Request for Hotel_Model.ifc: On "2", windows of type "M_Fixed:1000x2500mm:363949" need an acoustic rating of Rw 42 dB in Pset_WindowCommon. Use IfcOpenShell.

First a look at what the model holds.

```python
import ifcopenshell
import ifcopenshell.util.element

model = ifcopenshell.open("Hotel_Model.ifc")
print(model.schema)
storey = next(s for s in model.by_type("IfcBuildingStorey") if s.Name == "2")
windows = [e for e in ifcopenshell.util.element.get_decomposition(storey) if e.is_a("IfcWindow")]
seen = {}
for e in windows:
    element_type = ifcopenshell.util.element.get_type(e)
    key = (element_type.Name if element_type != e and element_type else None, ifcopenshell.util.element.get_pset(e, "Pset_WindowCommon", "AcousticRating"))
    seen[key] = seen.get(key, 0) + 1
for (name, value), count in sorted(seen.items(), key=str):
    print(count, "x", name, "|", value)
```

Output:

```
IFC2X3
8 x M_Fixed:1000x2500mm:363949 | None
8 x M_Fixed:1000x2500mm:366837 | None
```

```python
import ifcopenshell
import ifcopenshell.api.pset
import ifcopenshell.util.element

model = ifcopenshell.open("Hotel_Model.ifc")

storey = next(s for s in model.by_type("IfcBuildingStorey") if s.Name == "2")
windows = [e for e in ifcopenshell.util.element.get_decomposition(storey) if e.is_a("IfcWindow")]

count = 0
for e in windows:
    element_type = ifcopenshell.util.element.get_type(e)
    if element_type in (None, e) or element_type.Name != "M_Fixed:1000x2500mm:363949":
        continue
    # add_pset returns the element's existing set when there is one.
    pset = ifcopenshell.api.pset.add_pset(model, product=e, name="Pset_WindowCommon")
    ifcopenshell.api.pset.edit_pset(model, pset=pset, properties={"AcousticRating": "Rw 42 dB"})
    count += 1

print(count, "windows updated")

model.write("Hotel_Model_edited.ifc")
```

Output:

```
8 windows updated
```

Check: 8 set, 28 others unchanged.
